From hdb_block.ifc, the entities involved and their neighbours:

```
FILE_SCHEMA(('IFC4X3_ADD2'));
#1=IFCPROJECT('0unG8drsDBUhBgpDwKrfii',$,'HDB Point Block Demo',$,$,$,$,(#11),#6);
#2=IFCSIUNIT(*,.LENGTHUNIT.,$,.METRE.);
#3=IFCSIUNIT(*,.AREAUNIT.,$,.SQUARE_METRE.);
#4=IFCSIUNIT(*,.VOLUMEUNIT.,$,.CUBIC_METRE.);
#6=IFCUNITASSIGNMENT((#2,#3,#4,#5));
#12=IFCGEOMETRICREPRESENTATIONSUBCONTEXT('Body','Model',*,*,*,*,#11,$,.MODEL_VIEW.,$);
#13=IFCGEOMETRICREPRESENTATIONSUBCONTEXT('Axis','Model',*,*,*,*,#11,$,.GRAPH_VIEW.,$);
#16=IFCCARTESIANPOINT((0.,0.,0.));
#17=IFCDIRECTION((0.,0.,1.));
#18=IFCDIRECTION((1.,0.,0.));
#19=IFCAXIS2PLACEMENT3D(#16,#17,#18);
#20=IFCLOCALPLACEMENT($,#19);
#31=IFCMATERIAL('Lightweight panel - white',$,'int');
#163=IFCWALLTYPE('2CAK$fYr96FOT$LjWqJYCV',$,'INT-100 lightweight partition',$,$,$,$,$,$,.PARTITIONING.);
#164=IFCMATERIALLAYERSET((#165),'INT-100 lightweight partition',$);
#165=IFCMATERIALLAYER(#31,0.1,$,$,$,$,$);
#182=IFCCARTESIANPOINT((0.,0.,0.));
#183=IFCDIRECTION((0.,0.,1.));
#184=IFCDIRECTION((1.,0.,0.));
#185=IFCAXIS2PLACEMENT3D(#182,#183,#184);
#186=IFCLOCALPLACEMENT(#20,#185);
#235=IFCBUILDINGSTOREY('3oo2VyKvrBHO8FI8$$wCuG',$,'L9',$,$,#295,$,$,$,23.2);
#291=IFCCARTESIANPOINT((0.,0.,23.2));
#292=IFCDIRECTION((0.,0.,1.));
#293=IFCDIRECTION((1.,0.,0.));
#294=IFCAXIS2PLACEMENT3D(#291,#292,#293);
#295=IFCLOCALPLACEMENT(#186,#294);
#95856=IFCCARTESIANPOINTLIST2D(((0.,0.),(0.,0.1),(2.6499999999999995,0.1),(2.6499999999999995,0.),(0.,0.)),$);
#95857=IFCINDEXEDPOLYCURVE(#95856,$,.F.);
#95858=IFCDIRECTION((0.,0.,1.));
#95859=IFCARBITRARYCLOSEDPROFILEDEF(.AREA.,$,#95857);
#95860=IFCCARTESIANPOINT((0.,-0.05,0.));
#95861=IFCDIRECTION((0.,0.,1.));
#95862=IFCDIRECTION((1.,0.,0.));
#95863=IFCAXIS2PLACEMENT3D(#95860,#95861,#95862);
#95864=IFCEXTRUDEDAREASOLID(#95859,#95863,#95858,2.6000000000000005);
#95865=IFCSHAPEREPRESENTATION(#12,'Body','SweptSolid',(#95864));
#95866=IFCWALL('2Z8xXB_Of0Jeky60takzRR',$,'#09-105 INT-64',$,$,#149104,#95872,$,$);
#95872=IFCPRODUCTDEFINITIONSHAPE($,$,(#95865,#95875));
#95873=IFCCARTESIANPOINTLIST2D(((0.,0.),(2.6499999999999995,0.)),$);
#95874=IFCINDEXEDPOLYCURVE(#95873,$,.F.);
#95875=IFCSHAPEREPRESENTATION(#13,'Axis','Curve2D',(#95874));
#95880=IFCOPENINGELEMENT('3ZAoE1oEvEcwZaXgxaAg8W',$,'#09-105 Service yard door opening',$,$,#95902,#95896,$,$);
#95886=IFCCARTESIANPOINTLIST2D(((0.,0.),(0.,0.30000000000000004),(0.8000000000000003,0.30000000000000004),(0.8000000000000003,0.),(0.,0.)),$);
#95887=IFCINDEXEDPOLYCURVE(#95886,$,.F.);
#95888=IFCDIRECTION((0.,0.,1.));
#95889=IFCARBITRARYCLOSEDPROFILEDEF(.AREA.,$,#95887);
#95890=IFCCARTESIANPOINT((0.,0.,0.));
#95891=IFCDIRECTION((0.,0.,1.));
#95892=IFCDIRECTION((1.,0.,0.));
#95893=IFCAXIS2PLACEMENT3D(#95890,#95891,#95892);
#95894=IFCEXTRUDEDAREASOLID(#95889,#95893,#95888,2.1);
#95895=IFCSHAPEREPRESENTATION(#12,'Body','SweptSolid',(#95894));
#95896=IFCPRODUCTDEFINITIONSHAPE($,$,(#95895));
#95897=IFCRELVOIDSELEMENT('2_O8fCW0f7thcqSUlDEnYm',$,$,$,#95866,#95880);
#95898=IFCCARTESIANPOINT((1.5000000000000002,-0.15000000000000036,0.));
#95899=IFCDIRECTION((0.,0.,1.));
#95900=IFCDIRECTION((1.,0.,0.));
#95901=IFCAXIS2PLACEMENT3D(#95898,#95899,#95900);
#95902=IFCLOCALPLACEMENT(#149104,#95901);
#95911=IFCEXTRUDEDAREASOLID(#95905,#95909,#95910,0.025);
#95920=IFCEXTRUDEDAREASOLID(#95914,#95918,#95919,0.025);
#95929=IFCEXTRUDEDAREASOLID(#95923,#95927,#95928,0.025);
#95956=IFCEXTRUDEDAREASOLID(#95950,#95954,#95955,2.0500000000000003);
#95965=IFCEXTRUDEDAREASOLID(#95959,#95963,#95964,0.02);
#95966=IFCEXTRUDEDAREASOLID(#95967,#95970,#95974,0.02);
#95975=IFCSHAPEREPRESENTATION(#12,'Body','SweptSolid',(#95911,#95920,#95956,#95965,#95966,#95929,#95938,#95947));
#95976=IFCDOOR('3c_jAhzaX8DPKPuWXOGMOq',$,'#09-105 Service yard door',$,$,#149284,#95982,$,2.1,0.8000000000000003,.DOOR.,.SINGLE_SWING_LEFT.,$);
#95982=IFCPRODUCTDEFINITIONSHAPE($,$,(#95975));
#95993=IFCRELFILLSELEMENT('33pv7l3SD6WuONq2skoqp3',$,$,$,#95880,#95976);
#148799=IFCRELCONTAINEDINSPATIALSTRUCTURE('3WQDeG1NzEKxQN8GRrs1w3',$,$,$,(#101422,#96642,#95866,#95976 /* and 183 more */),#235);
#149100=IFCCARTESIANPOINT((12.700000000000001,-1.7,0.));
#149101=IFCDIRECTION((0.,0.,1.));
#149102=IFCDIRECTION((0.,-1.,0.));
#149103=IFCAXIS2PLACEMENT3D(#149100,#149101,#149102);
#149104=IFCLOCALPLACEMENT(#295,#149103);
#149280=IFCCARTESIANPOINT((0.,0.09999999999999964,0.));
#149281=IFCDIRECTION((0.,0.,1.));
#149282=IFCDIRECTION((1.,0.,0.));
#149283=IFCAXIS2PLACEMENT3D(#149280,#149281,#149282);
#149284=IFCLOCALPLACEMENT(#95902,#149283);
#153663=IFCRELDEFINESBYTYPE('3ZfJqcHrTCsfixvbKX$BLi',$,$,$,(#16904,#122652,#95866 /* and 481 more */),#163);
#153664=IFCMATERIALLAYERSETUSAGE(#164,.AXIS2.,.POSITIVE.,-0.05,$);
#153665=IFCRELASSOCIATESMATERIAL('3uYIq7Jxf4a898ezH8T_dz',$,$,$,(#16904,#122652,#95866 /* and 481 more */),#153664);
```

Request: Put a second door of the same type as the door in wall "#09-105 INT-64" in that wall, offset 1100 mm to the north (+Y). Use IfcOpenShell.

```python
import ifcopenshell
import ifcopenshell.api.feature
import ifcopenshell.api.geometry
import ifcopenshell.api.root
import ifcopenshell.geom
import ifcopenshell.util.element
import ifcopenshell.util.placement
import ifcopenshell.util.shape

model = ifcopenshell.open("hdb_block.ifc")
settings = ifcopenshell.geom.settings()


def volume(element):
    """Net volume in cubic metres, openings subtracted."""
    shape = ifcopenshell.geom.create_shape(settings, element)
    return ifcopenshell.util.shape.get_volume(shape.geometry)


door = model.by_guid("3c_jAhzaX8DPKPuWXOGMOq")
opening = door.FillsVoids[0].RelatingOpeningElement
wall = opening.VoidsElements[0].RelatingBuildingElement
before = volume(wall)
shift = ifcopenshell.util.placement.get_local_placement(wall.ObjectPlacement)[:3, 0] * -1.1

# copy_class copies the void relationship, type, container and properties, but no geometry.
new_opening = ifcopenshell.api.root.copy_class(model, product=opening)
new_opening.Representation = ifcopenshell.util.element.copy_deep(
    model, opening.Representation, exclude=["IfcGeometricRepresentationContext", "IfcRepresentationMap"]
)
new_door = ifcopenshell.api.root.copy_class(model, product=door)
new_door.Representation = ifcopenshell.util.element.copy_deep(
    model, door.Representation, exclude=["IfcGeometricRepresentationContext", "IfcRepresentationMap"]
)
ifcopenshell.api.feature.add_filling(model, opening=new_opening, element=new_door)

for old, new in ((opening, new_opening), (door, new_door)):
    matrix = ifcopenshell.util.placement.get_local_placement(old.ObjectPlacement)
    matrix[:3, 3] += shift
    ifcopenshell.api.geometry.edit_object_placement(model, product=new, matrix=matrix, is_si=False)

after = volume(wall)

print(f"wall volume {before:.3f} -> {after:.3f} m3")

model.write("hdb_block_edited.ifc")
```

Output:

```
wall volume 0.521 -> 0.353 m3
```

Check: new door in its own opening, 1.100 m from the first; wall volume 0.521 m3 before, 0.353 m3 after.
